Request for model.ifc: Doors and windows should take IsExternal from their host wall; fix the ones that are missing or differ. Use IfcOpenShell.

First a look at what the model holds.

```python
import ifcopenshell
import ifcopenshell.util.element

model = ifcopenshell.open("model.ifc")
print(model.schema)
seen = {}
for e in model.by_type("IfcDoor") + model.by_type("IfcWindow"):
    if not e.FillsVoids:
        continue
    host = e.FillsVoids[0].RelatingOpeningElement.VoidsElements[0].RelatingBuildingElement
    own = ifcopenshell.util.element.get_pset(e, f"Pset_{e.is_a()[3:].removesuffix('StandardCase')}Common", "IsExternal")
    wall = ifcopenshell.util.element.get_pset(host, "Pset_WallCommon", "IsExternal")
    seen[e.is_a(), own, wall] = seen.get((e.is_a(), own, wall), 0) + 1
for (cls, own, wall), count in sorted(seen.items(), key=str):
    print(count, cls, "IsExternal:", own, "| host wall:", wall)
```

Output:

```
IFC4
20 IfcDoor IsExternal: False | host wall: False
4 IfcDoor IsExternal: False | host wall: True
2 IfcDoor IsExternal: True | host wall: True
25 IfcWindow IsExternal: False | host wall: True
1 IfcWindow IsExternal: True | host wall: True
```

```python
import ifcopenshell
import ifcopenshell.api.pset
import ifcopenshell.util.element

model = ifcopenshell.open("model.ifc")

count = 0
for ifc_class, pset_name in (("IfcDoor", "Pset_DoorCommon"), ("IfcWindow", "Pset_WindowCommon")):
    for e in model.by_type(ifc_class):
        if not e.FillsVoids:
            continue
        host = e.FillsVoids[0].RelatingOpeningElement.VoidsElements[0].RelatingBuildingElement
        external = ifcopenshell.util.element.get_pset(host, "Pset_WallCommon", "IsExternal")
        if external is None or ifcopenshell.util.element.get_pset(e, pset_name, "IsExternal") == external:
            continue
        pset = ifcopenshell.api.pset.add_pset(model, product=e, name=pset_name)
        ifcopenshell.api.pset.edit_pset(model, pset=pset, properties={"IsExternal": external})
        count += 1

print(count, "updated")

model.write("model_updated.ifc")
```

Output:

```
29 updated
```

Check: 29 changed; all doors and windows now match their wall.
